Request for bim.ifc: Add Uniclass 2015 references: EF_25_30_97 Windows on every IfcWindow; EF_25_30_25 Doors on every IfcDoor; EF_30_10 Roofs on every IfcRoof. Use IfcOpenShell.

First a look at what the model holds.

```python
import ifcopenshell

model = ifcopenshell.open("bim.ifc")
print(model.schema)
print("classifications:", [c.Name for c in model.by_type("IfcClassification")])
for ifc_class in ("IfcDoor", "IfcRoof", "IfcStair", "IfcWall", "IfcWindow"):
    print(ifc_class, len(model.by_type(ifc_class)))
```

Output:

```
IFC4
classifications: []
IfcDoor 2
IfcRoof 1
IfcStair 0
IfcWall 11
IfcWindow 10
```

```python
import ifcopenshell
import ifcopenshell.api.classification

model = ifcopenshell.open("bim.ifc")

system = ifcopenshell.api.classification.add_classification(model, classification="Uniclass 2015")

codes = {
    "IfcWindow": ("EF_25_30_97", "Windows"),
    "IfcDoor": ("EF_25_30_25", "Doors"),
    "IfcRoof": ("EF_30_10", "Roofs"),
}
for ifc_class, (code, name) in codes.items():
    products = model.by_type(ifc_class)
    ifcopenshell.api.classification.add_reference(
        model, products=products, classification=system, identification=code, name=name
    )
    print(code, len(products))

model.write("bim_v2.ifc")
```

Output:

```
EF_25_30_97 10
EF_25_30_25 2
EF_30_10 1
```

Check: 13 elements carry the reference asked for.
